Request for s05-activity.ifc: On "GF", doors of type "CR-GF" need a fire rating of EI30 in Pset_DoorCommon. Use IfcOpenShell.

First a look at what the model holds.

```python
import ifcopenshell
import ifcopenshell.util.element

model = ifcopenshell.open("s05-activity.ifc")
print(model.schema)
storey = next(s for s in model.by_type("IfcBuildingStorey") if s.Name == "GF")
doors = [e for e in ifcopenshell.util.element.get_decomposition(storey) if e.is_a("IfcDoor")]
seen = {}
for e in doors:
    element_type = ifcopenshell.util.element.get_type(e)
    key = (element_type.Name if element_type != e and element_type else None, ifcopenshell.util.element.get_pset(e, "Pset_DoorCommon", "FireRating"))
    seen[key] = seen.get(key, 0) + 1
for (name, value), count in sorted(seen.items(), key=str):
    print(count, "x", name, "|", value)
```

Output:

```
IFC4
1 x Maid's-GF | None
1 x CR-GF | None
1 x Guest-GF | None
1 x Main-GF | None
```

```python
import ifcopenshell
import ifcopenshell.api.pset
import ifcopenshell.util.element

model = ifcopenshell.open("s05-activity.ifc")

storey = next(s for s in model.by_type("IfcBuildingStorey") if s.Name == "GF")
doors = [e for e in ifcopenshell.util.element.get_decomposition(storey) if e.is_a("IfcDoor")]

count = 0
for e in doors:
    element_type = ifcopenshell.util.element.get_type(e)
    if element_type in (None, e) or element_type.Name != "CR-GF":
        continue
    # add_pset returns the element's existing set when there is one.
    pset = ifcopenshell.api.pset.add_pset(model, product=e, name="Pset_DoorCommon")
    ifcopenshell.api.pset.edit_pset(model, pset=pset, properties={"FireRating": "EI30"})
    count += 1

print(count, "doors updated")

model.write("s05-activity_v2.ifc")
```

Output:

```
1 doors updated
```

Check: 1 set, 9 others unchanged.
